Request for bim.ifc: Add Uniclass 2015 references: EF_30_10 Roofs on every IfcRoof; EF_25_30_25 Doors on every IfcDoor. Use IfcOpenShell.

First a look at what the model holds.

```python
import ifcopenshell

model = ifcopenshell.open("bim.ifc")
print(model.schema)
print("classifications:", [c.Name for c in model.by_type("IfcClassification")])
for ifc_class in ("IfcDoor", "IfcRoof", "IfcStair", "IfcWall", "IfcWindow"):
    print(ifc_class, len(model.by_type(ifc_class)))
```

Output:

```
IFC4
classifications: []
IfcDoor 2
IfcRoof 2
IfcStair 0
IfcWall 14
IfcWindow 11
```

```python
import ifcopenshell
import ifcopenshell.api.classification

model = ifcopenshell.open("bim.ifc")

system = ifcopenshell.api.classification.add_classification(model, classification="Uniclass 2015")

codes = {
    "IfcRoof": ("EF_30_10", "Roofs"),
    "IfcDoor": ("EF_25_30_25", "Doors"),
}
for ifc_class, (code, name) in codes.items():
    products = model.by_type(ifc_class)
    ifcopenshell.api.classification.add_reference(
        model, products=products, classification=system, identification=code, name=name
    )
    print(code, len(products))

model.write("bim-out.ifc")
```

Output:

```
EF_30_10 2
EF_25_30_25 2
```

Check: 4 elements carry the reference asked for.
